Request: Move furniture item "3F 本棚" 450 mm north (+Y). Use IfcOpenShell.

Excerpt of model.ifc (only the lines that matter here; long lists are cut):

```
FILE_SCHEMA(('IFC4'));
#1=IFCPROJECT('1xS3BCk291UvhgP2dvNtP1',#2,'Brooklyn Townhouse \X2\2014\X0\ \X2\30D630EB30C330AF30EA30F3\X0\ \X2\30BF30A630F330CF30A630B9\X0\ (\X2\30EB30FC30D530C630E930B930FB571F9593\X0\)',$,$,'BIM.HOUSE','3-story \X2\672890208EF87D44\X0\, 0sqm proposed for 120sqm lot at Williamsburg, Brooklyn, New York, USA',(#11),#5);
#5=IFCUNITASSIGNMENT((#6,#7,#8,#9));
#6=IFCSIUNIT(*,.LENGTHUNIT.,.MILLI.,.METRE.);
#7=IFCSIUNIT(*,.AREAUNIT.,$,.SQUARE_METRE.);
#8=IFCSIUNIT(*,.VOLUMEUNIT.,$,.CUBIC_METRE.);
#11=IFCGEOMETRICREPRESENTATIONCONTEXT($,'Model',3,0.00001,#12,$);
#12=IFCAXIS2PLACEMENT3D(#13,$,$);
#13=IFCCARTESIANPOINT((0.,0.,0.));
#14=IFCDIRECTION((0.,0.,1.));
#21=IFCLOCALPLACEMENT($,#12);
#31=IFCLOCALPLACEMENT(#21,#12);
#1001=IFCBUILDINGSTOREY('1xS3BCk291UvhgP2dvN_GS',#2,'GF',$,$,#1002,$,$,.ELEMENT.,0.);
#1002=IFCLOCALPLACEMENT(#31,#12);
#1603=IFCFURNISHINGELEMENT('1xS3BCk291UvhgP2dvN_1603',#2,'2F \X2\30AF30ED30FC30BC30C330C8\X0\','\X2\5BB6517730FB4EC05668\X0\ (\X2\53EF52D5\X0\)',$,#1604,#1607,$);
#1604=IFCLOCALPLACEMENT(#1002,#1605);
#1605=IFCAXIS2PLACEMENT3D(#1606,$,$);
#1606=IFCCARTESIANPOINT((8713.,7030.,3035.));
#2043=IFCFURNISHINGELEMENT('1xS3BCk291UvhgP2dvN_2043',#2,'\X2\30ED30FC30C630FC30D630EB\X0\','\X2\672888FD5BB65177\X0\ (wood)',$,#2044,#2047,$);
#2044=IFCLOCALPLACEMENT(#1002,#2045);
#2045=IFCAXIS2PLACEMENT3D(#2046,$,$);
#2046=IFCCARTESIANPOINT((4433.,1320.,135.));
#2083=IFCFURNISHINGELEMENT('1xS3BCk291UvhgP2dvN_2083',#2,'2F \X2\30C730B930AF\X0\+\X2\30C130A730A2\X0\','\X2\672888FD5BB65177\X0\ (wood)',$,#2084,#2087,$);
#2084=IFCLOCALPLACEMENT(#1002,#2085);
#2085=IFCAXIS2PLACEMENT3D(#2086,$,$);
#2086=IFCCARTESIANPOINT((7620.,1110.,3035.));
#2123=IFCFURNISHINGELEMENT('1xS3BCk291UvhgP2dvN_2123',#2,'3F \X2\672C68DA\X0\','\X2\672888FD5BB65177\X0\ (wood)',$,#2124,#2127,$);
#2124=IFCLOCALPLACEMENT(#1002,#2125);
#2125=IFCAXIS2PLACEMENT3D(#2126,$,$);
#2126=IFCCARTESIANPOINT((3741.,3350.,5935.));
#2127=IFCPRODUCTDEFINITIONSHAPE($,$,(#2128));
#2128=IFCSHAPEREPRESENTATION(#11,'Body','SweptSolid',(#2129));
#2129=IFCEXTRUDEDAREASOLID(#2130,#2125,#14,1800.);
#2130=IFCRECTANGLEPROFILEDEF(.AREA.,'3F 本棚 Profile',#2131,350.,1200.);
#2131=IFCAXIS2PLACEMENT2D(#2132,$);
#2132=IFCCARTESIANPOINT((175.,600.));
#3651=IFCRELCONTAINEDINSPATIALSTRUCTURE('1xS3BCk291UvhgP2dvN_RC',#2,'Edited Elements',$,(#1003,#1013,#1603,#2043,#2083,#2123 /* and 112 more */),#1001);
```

```python
import ifcopenshell
import ifcopenshell.api.geometry
import ifcopenshell.util.placement
import ifcopenshell.util.unit

model = ifcopenshell.open("model.ifc")
unit_scale = ifcopenshell.util.unit.calculate_unit_scale(model)

item = model.by_guid("1xS3BCk291UvhgP2dvN_2123")
matrix = ifcopenshell.util.placement.get_local_placement(item.ObjectPlacement)
matrix[1, 3] += 0.45 / unit_scale
ifcopenshell.api.geometry.edit_object_placement(model, product=item, matrix=matrix, is_si=False)

print(ifcopenshell.util.placement.get_local_placement(item.ObjectPlacement).round(3) + 0.0)

model.write("model_rev.ifc")
```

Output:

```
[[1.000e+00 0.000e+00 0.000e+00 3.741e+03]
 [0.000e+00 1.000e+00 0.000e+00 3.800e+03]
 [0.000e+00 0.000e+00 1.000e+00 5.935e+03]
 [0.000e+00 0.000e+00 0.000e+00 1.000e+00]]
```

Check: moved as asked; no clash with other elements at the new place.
